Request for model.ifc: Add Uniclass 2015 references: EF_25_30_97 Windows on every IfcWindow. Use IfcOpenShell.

First a look at what the model holds.

```python
import ifcopenshell

model = ifcopenshell.open("model.ifc")
print(model.schema)
print("classifications:", [c.Name for c in model.by_type("IfcClassification")])
for ifc_class in ("IfcDoor", "IfcRoof", "IfcStair", "IfcWall", "IfcWindow"):
    print(ifc_class, len(model.by_type(ifc_class)))
```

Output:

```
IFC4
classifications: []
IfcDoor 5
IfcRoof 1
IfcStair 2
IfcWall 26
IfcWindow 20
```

```python
import ifcopenshell
import ifcopenshell.api.classification

model = ifcopenshell.open("model.ifc")

system = ifcopenshell.api.classification.add_classification(model, classification="Uniclass 2015")

codes = {
    "IfcWindow": ("EF_25_30_97", "Windows"),
}
for ifc_class, (code, name) in codes.items():
    products = model.by_type(ifc_class)
    ifcopenshell.api.classification.add_reference(
        model, products=products, classification=system, identification=code, name=name
    )
    print(code, len(products))

model.write("model_updated.ifc")
```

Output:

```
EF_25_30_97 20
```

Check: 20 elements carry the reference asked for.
